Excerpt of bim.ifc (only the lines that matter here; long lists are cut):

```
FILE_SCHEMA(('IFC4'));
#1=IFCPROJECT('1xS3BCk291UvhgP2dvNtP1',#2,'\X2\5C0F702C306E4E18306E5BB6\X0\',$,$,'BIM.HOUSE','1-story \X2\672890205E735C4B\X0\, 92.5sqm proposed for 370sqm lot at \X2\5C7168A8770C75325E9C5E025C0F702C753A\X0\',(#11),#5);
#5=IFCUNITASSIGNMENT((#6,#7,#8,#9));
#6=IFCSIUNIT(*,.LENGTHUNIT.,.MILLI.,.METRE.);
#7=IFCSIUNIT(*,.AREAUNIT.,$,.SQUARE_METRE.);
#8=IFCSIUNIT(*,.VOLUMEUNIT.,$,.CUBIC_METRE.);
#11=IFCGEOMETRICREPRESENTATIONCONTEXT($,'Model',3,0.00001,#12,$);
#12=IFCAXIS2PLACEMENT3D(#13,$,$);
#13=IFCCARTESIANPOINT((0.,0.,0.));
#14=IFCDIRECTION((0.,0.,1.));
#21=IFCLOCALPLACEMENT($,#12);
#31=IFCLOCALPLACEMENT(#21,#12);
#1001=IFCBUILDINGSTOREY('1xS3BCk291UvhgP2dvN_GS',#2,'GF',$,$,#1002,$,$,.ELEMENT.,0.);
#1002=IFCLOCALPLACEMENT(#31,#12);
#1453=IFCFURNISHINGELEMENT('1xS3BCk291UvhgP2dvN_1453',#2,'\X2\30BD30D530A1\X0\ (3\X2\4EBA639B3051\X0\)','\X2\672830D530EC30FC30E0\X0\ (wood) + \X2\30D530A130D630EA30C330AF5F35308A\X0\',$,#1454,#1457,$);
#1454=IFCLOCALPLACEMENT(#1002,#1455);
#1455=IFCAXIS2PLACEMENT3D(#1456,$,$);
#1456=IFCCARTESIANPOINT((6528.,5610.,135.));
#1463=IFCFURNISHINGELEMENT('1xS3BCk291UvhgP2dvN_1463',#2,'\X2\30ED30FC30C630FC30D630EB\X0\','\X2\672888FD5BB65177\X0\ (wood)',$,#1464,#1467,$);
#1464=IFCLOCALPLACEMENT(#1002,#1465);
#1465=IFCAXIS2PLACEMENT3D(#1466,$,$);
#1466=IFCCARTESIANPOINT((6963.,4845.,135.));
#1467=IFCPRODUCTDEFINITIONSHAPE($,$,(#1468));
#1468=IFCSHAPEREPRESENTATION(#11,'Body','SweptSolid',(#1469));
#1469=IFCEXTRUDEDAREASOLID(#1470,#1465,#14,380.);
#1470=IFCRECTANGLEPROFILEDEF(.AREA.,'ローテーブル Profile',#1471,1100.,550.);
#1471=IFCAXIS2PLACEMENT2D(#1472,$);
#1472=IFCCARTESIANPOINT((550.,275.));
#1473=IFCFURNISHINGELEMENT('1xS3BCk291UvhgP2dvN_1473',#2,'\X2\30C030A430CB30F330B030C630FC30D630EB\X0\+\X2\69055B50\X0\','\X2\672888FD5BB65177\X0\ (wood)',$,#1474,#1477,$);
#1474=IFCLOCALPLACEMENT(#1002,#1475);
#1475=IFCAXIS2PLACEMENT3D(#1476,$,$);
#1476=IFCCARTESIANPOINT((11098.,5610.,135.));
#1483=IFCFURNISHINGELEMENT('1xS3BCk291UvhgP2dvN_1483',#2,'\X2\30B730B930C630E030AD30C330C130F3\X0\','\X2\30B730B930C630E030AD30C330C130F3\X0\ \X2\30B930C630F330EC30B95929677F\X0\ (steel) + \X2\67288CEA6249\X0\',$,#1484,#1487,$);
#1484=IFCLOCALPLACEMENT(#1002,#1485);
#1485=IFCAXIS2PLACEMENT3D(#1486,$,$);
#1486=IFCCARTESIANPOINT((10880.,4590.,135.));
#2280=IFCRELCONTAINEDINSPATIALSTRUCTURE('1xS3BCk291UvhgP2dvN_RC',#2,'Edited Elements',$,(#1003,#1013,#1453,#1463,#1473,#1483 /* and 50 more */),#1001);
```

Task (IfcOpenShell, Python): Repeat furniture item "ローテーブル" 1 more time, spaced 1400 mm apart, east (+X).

```python
import numpy as np
import ifcopenshell
import ifcopenshell.api.geometry
import ifcopenshell.api.root
import ifcopenshell.util.element
import ifcopenshell.util.placement

model = ifcopenshell.open("bim.ifc")


def reuse_history(source, copy):
    """copy_class also copies each property set's owner history, people and application; keep the originals."""
    for rel in copy.IsDefinedBy:
        if rel.is_a("IfcRelDefinesByProperties") and (history := rel.RelatingPropertyDefinition.OwnerHistory):
            rel.RelatingPropertyDefinition.OwnerHistory = source.OwnerHistory
            ifcopenshell.util.element.remove_deep2(model, history)


source = model.by_id(1463)
base = ifcopenshell.util.placement.get_local_placement(source.ObjectPlacement)
step = np.array([1.0, 0.0, 0.0]) * 1400.0

for i in range(1, 2):
    copy = ifcopenshell.api.root.copy_class(model, product=source)
    copy.Representation = ifcopenshell.util.element.copy_deep(
        model, source.Representation, exclude=["IfcGeometricRepresentationContext", "IfcRepresentationMap"]
    )
    reuse_history(source, copy)
    matrix = base.copy()
    matrix[:3, 3] += i * step
    print("added at", matrix[:3, 3].round(3) + 0.0)
    ifcopenshell.api.geometry.edit_object_placement(model, product=copy, matrix=matrix, is_si=False)

model.write("bim_edited.ifc")
```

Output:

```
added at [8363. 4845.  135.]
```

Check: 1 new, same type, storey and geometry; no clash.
